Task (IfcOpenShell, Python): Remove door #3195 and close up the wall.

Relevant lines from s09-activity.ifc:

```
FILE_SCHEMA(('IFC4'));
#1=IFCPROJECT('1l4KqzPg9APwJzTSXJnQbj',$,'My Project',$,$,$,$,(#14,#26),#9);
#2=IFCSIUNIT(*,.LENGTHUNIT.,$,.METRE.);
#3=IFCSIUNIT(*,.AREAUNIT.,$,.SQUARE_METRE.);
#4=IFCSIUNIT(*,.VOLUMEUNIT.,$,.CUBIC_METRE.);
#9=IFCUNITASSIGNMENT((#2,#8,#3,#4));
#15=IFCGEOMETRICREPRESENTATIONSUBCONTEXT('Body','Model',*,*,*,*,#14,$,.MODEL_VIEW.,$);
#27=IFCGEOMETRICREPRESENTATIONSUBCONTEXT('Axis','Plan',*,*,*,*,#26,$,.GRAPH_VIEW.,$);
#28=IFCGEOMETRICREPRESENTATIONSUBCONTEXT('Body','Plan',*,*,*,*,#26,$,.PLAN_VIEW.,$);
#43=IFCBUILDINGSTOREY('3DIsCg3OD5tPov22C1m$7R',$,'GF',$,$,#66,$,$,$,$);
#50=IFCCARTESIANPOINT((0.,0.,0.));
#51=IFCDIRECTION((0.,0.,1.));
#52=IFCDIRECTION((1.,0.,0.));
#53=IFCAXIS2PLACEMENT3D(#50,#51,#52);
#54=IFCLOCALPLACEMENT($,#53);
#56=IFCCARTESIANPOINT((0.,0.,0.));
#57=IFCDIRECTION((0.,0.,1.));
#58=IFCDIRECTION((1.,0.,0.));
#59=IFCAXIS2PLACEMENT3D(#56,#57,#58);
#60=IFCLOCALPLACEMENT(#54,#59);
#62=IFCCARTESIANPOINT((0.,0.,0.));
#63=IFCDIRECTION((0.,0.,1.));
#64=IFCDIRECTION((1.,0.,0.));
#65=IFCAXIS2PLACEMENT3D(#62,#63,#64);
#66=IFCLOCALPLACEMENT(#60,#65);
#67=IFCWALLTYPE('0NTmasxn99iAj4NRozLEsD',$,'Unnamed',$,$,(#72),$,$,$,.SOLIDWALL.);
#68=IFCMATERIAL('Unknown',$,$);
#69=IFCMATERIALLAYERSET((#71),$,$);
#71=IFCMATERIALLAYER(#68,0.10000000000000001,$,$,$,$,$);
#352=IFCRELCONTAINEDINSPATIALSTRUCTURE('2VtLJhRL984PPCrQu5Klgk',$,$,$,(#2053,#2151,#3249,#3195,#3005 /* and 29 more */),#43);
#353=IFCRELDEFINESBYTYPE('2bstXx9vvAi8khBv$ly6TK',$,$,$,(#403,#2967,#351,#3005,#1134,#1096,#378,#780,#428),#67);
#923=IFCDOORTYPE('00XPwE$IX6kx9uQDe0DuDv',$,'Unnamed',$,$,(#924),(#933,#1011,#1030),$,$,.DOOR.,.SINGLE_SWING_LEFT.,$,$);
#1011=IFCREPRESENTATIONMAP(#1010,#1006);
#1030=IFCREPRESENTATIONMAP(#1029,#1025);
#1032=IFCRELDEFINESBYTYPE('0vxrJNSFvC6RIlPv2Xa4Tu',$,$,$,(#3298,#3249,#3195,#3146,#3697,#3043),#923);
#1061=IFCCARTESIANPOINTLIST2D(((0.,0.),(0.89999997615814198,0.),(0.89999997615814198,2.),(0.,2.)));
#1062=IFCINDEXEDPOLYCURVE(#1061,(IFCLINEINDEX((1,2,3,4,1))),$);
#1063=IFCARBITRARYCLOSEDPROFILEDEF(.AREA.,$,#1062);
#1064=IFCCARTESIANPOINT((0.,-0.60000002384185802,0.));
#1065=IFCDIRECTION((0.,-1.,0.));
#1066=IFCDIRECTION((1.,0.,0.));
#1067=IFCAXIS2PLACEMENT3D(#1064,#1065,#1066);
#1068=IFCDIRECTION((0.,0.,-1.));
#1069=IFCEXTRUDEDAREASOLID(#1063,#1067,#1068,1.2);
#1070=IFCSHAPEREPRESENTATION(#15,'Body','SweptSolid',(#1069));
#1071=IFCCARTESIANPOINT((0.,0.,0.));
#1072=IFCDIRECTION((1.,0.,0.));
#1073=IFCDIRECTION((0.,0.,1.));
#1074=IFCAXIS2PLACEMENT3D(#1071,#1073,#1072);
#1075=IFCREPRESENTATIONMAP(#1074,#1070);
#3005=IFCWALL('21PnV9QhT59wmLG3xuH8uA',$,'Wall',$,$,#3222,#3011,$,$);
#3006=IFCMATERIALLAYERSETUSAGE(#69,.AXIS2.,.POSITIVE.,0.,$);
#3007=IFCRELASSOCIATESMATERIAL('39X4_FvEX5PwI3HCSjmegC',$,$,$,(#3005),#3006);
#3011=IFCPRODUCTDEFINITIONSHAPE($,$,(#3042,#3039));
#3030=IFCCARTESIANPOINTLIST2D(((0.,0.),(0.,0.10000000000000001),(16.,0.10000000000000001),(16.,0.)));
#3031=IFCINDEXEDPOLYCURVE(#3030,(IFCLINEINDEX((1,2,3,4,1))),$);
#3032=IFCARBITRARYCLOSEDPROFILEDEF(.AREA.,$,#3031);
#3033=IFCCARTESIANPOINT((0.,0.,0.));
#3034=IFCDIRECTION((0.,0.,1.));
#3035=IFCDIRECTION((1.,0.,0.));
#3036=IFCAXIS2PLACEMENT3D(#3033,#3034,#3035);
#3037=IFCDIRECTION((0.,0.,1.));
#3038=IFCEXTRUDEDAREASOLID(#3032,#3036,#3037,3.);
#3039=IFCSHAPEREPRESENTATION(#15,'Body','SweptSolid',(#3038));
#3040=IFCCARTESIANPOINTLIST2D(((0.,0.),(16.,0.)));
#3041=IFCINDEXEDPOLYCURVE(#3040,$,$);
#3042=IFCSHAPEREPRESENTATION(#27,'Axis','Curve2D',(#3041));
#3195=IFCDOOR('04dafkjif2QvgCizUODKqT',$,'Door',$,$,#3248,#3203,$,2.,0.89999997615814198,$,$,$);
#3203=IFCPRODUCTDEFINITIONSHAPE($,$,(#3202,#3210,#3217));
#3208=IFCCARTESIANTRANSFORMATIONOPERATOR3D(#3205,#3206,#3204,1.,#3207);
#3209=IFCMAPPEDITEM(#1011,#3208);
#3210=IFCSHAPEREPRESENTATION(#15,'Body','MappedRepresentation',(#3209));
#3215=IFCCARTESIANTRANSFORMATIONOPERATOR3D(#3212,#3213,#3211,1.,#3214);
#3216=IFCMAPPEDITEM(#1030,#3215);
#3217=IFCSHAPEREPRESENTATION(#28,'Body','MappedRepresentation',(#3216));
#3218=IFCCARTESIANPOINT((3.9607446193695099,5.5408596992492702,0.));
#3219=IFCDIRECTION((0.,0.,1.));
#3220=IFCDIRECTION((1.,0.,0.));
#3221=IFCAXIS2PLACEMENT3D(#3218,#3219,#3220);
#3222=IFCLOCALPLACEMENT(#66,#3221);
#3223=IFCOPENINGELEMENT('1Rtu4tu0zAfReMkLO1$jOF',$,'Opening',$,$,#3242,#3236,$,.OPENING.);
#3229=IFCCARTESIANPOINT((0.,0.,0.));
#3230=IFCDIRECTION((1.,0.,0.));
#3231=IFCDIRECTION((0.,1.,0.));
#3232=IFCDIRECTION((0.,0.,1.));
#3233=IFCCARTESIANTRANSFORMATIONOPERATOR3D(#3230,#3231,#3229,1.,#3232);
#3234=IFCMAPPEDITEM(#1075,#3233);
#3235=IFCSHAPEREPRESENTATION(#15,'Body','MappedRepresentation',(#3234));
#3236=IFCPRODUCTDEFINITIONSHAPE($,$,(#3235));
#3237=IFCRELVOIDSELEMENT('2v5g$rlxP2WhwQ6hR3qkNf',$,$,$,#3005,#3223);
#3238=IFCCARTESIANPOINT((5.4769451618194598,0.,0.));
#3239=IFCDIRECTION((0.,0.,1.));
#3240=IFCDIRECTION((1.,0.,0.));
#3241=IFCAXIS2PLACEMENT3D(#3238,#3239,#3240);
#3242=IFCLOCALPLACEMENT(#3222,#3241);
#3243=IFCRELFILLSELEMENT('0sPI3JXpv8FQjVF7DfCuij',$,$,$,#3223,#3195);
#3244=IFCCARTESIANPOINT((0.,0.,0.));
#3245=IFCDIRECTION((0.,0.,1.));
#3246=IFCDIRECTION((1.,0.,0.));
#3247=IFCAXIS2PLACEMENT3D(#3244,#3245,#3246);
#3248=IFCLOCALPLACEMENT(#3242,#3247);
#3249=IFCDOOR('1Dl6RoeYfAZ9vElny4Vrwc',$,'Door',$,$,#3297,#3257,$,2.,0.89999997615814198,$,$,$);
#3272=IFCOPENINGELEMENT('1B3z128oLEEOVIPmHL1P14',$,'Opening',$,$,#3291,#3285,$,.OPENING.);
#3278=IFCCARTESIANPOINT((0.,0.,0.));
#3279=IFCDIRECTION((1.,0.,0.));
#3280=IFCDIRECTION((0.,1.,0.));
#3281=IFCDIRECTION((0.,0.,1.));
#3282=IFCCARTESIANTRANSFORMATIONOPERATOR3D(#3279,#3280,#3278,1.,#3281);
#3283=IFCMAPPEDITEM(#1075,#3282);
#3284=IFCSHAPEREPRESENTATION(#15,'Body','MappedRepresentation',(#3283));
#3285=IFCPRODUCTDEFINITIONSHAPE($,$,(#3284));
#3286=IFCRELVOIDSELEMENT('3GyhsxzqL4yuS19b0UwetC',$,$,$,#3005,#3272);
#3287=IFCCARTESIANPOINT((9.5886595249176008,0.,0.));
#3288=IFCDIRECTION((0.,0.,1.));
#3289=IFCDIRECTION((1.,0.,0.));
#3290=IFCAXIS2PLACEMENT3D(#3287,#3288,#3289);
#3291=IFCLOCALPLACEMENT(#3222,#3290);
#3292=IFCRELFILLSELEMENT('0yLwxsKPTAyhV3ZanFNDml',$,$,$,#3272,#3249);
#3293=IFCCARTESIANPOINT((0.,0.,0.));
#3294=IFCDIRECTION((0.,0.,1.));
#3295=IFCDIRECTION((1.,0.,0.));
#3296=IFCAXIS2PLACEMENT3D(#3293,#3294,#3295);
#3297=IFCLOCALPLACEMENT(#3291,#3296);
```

```python
import ifcopenshell
import ifcopenshell.api.feature
import ifcopenshell.api.root
import ifcopenshell.geom
import ifcopenshell.util.shape

model = ifcopenshell.open("s09-activity.ifc")
settings = ifcopenshell.geom.settings()


def volume(element):
    """Net volume in cubic metres, openings subtracted."""
    shape = ifcopenshell.geom.create_shape(settings, element)
    return ifcopenshell.util.shape.get_volume(shape.geometry)


door = model.by_guid("04dafkjif2QvgCizUODKqT")
opening = door.FillsVoids[0].RelatingOpeningElement
wall = opening.VoidsElements[0].RelatingBuildingElement
before = volume(wall)

ifcopenshell.api.root.remove_product(model, product=door)
ifcopenshell.api.feature.remove_feature(model, feature=opening)

after = volume(wall)

print(f"wall volume {before:.3f} -> {after:.3f} m3")

model.write("s09-activity_updated.ifc")
```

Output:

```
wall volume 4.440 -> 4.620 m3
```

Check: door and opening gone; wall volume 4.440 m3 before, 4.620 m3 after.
